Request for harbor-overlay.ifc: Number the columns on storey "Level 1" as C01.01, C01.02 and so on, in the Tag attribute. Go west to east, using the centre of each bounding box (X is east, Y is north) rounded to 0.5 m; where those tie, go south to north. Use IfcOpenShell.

First a look at what the model holds.

```python
import ifcopenshell
import ifcopenshell.util.element
import ifcopenshell.util.placement

model = ifcopenshell.open("harbor-overlay.ifc")
print(model.schema)
storey = next(s for s in model.by_type("IfcBuildingStorey") if s.Name == "Level 1")
columns = [e for e in ifcopenshell.util.element.get_decomposition(storey) if e.is_a("IfcColumn")]
for e in sorted(columns, key=lambda e: e.id()):
    origin = ifcopenshell.util.placement.get_local_placement(e.ObjectPlacement)[:3, 3]
    print(e.id(), e.Tag, e.Name, origin.round(2) + 0.0, sep=" | ")
```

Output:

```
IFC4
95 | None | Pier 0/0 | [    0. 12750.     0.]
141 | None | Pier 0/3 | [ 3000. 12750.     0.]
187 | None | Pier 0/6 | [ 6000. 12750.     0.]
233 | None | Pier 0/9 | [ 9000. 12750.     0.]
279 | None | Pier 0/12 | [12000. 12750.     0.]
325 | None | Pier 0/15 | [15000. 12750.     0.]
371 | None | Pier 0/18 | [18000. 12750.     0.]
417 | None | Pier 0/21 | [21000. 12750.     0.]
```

```python
import ifcopenshell
import ifcopenshell.geom
import ifcopenshell.util.element
import ifcopenshell.util.shape

model = ifcopenshell.open("harbor-overlay.ifc")
settings = ifcopenshell.geom.settings()
settings.set("use-world-coords", True)


def centre(element):
    shape = ifcopenshell.geom.create_shape(settings, element)
    return ifcopenshell.util.shape.get_bbox_centroid(shape.geometry)


storey = next(s for s in model.by_type("IfcBuildingStorey") if s.Name == "Level 1")
columns = [e for e in ifcopenshell.util.element.get_decomposition(storey) if e.is_a("IfcColumn")]

# Insertion points can sit at a corner or the storey origin, so sort by the geometry (in metres).
centres = {e: centre(e) for e in columns}
columns.sort(key=lambda e: (round(centres[e][0] / 0.5), centres[e][1]))

for i, e in enumerate(columns, start=1):
    number = f"C01.{i:02d}"
    e.Tag = number
    print(e.id(), number)

model.write("harbor-overlay_rev.ifc")
```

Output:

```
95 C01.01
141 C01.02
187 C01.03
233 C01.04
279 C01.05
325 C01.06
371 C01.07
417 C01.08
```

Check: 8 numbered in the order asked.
